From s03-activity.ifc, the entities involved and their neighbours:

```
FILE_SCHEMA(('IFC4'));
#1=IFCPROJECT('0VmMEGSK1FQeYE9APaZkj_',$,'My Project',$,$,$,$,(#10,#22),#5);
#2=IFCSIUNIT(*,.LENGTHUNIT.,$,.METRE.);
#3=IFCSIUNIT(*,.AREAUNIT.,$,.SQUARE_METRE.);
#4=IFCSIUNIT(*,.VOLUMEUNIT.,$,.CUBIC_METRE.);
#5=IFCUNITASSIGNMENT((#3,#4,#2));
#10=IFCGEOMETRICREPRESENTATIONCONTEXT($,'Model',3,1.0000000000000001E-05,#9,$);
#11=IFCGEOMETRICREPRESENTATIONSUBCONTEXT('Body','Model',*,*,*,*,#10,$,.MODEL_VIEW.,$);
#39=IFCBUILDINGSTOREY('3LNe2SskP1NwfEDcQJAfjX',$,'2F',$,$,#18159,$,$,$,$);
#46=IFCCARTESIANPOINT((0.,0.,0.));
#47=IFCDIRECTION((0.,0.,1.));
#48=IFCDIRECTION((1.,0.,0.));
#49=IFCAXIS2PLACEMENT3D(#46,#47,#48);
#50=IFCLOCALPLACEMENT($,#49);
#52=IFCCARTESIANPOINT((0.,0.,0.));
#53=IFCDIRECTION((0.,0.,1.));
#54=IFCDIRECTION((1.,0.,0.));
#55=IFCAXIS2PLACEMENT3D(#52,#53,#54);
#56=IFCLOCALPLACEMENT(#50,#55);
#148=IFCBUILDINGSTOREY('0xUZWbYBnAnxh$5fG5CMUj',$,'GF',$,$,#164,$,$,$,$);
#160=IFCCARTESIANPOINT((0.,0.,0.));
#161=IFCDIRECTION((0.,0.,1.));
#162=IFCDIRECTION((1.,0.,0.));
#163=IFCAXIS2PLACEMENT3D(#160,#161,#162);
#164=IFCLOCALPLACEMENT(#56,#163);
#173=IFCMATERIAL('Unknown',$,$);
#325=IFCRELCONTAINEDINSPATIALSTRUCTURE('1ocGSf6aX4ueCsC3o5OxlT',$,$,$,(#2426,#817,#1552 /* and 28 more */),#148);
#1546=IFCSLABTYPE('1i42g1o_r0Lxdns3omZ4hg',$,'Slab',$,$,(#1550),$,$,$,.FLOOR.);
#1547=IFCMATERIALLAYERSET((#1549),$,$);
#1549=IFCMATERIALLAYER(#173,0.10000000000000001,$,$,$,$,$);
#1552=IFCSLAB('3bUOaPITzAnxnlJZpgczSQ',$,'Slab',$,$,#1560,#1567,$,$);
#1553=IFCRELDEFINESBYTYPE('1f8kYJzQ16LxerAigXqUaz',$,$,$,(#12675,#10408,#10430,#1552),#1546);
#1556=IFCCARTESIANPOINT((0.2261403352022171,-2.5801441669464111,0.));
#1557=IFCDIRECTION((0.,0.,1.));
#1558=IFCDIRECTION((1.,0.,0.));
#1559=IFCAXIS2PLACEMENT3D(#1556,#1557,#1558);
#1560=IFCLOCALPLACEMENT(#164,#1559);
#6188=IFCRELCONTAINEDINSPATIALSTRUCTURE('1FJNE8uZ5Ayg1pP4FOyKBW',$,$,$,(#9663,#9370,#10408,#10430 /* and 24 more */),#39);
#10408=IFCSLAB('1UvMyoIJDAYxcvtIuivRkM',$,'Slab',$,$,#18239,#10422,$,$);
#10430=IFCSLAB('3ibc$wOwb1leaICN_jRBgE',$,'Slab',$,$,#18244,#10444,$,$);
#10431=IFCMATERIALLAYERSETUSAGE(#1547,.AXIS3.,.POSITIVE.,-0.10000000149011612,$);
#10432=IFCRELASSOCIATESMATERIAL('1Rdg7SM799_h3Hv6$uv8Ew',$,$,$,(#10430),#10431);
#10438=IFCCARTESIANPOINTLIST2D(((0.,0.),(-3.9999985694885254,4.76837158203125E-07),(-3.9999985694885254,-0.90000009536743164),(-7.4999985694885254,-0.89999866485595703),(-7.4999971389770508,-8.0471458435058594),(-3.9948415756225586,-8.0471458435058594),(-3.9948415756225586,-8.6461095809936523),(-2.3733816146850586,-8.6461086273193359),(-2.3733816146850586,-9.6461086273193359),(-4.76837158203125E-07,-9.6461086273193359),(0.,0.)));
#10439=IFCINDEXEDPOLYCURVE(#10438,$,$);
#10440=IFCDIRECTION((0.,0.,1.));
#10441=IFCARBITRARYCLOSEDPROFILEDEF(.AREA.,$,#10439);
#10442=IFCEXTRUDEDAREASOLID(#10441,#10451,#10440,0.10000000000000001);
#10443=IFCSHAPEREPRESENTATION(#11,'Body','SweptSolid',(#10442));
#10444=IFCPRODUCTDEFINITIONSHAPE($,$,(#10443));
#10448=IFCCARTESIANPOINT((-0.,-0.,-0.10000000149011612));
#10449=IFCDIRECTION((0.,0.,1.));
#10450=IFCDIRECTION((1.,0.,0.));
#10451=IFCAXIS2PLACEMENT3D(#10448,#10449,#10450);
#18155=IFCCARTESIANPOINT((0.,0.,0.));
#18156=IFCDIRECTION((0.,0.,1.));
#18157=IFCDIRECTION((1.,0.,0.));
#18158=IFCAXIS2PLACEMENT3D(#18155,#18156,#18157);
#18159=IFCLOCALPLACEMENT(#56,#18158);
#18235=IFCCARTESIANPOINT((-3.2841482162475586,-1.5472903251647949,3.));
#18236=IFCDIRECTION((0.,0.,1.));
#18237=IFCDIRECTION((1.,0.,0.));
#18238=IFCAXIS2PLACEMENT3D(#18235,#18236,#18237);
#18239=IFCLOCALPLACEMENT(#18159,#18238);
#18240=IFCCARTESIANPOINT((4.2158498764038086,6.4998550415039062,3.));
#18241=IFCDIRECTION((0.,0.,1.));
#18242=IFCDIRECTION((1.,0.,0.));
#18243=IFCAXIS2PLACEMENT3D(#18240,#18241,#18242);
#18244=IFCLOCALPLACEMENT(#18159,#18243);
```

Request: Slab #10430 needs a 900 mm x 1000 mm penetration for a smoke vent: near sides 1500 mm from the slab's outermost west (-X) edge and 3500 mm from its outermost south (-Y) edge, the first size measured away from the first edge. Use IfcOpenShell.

```python
import numpy as np
import ifcopenshell
import ifcopenshell.api.feature
import ifcopenshell.api.geometry
import ifcopenshell.api.root
import ifcopenshell.geom
import ifcopenshell.util.placement
import ifcopenshell.util.representation
import ifcopenshell.util.shape
import ifcopenshell.util.unit

model = ifcopenshell.open("s03-activity.ifc")
unit_scale = ifcopenshell.util.unit.calculate_unit_scale(model)
settings = ifcopenshell.geom.settings()


def volume(element):
    """Net volume in cubic metres, openings subtracted."""
    shape = ifcopenshell.geom.create_shape(settings, element)
    return ifcopenshell.util.shape.get_volume(shape.geometry)


slab = model.by_guid("3ibc$wOwb1leaICN_jRBgE")
before = volume(slab)

# Extent in the slab's own axes, in metres. The edges named are its -X and -Y sides.
slab_shape = ifcopenshell.geom.create_shape(settings, slab)
vertices = ifcopenshell.util.shape.get_vertices(slab_shape.geometry)
x_min, y_min, bottom = vertices.min(axis=0)
top = vertices[:, 2].max()

opening = ifcopenshell.api.root.create_entity(model, ifc_class="IfcOpeningElement", name="Smoke vent opening", predefined_type="OPENING")
context = ifcopenshell.util.representation.get_context(model, "Model", "Body", "MODEL_VIEW")
width, depth = 0.9, 1
outline = [(0.0, 0.0), (width, 0.0), (width, depth), (0.0, depth), (0.0, 0.0)]
# Overshoot both faces by 50 mm so the cut is clean.
shape = ifcopenshell.api.geometry.add_slab_representation(
    model, context=context, depth=top - bottom + 0.1, polyline=outline
)
ifcopenshell.api.geometry.assign_representation(model, product=opening, representation=shape)

matrix = ifcopenshell.util.placement.get_local_placement(slab.ObjectPlacement)
matrix[:, 3] = matrix @ np.append(np.array([x_min + 1.5, y_min + 3.5, bottom - 0.05]) / unit_scale, 1.0)
ifcopenshell.api.geometry.edit_object_placement(model, product=opening, matrix=matrix, is_si=False)
ifcopenshell.api.feature.add_feature(model, feature=opening, element=slab)

after = volume(slab)

print(f"slab volume {before:.3f} -> {after:.3f} m3")

model.write("s03-activity_updated.ifc")
```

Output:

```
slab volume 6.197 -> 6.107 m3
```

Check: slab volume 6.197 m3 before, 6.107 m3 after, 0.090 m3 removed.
